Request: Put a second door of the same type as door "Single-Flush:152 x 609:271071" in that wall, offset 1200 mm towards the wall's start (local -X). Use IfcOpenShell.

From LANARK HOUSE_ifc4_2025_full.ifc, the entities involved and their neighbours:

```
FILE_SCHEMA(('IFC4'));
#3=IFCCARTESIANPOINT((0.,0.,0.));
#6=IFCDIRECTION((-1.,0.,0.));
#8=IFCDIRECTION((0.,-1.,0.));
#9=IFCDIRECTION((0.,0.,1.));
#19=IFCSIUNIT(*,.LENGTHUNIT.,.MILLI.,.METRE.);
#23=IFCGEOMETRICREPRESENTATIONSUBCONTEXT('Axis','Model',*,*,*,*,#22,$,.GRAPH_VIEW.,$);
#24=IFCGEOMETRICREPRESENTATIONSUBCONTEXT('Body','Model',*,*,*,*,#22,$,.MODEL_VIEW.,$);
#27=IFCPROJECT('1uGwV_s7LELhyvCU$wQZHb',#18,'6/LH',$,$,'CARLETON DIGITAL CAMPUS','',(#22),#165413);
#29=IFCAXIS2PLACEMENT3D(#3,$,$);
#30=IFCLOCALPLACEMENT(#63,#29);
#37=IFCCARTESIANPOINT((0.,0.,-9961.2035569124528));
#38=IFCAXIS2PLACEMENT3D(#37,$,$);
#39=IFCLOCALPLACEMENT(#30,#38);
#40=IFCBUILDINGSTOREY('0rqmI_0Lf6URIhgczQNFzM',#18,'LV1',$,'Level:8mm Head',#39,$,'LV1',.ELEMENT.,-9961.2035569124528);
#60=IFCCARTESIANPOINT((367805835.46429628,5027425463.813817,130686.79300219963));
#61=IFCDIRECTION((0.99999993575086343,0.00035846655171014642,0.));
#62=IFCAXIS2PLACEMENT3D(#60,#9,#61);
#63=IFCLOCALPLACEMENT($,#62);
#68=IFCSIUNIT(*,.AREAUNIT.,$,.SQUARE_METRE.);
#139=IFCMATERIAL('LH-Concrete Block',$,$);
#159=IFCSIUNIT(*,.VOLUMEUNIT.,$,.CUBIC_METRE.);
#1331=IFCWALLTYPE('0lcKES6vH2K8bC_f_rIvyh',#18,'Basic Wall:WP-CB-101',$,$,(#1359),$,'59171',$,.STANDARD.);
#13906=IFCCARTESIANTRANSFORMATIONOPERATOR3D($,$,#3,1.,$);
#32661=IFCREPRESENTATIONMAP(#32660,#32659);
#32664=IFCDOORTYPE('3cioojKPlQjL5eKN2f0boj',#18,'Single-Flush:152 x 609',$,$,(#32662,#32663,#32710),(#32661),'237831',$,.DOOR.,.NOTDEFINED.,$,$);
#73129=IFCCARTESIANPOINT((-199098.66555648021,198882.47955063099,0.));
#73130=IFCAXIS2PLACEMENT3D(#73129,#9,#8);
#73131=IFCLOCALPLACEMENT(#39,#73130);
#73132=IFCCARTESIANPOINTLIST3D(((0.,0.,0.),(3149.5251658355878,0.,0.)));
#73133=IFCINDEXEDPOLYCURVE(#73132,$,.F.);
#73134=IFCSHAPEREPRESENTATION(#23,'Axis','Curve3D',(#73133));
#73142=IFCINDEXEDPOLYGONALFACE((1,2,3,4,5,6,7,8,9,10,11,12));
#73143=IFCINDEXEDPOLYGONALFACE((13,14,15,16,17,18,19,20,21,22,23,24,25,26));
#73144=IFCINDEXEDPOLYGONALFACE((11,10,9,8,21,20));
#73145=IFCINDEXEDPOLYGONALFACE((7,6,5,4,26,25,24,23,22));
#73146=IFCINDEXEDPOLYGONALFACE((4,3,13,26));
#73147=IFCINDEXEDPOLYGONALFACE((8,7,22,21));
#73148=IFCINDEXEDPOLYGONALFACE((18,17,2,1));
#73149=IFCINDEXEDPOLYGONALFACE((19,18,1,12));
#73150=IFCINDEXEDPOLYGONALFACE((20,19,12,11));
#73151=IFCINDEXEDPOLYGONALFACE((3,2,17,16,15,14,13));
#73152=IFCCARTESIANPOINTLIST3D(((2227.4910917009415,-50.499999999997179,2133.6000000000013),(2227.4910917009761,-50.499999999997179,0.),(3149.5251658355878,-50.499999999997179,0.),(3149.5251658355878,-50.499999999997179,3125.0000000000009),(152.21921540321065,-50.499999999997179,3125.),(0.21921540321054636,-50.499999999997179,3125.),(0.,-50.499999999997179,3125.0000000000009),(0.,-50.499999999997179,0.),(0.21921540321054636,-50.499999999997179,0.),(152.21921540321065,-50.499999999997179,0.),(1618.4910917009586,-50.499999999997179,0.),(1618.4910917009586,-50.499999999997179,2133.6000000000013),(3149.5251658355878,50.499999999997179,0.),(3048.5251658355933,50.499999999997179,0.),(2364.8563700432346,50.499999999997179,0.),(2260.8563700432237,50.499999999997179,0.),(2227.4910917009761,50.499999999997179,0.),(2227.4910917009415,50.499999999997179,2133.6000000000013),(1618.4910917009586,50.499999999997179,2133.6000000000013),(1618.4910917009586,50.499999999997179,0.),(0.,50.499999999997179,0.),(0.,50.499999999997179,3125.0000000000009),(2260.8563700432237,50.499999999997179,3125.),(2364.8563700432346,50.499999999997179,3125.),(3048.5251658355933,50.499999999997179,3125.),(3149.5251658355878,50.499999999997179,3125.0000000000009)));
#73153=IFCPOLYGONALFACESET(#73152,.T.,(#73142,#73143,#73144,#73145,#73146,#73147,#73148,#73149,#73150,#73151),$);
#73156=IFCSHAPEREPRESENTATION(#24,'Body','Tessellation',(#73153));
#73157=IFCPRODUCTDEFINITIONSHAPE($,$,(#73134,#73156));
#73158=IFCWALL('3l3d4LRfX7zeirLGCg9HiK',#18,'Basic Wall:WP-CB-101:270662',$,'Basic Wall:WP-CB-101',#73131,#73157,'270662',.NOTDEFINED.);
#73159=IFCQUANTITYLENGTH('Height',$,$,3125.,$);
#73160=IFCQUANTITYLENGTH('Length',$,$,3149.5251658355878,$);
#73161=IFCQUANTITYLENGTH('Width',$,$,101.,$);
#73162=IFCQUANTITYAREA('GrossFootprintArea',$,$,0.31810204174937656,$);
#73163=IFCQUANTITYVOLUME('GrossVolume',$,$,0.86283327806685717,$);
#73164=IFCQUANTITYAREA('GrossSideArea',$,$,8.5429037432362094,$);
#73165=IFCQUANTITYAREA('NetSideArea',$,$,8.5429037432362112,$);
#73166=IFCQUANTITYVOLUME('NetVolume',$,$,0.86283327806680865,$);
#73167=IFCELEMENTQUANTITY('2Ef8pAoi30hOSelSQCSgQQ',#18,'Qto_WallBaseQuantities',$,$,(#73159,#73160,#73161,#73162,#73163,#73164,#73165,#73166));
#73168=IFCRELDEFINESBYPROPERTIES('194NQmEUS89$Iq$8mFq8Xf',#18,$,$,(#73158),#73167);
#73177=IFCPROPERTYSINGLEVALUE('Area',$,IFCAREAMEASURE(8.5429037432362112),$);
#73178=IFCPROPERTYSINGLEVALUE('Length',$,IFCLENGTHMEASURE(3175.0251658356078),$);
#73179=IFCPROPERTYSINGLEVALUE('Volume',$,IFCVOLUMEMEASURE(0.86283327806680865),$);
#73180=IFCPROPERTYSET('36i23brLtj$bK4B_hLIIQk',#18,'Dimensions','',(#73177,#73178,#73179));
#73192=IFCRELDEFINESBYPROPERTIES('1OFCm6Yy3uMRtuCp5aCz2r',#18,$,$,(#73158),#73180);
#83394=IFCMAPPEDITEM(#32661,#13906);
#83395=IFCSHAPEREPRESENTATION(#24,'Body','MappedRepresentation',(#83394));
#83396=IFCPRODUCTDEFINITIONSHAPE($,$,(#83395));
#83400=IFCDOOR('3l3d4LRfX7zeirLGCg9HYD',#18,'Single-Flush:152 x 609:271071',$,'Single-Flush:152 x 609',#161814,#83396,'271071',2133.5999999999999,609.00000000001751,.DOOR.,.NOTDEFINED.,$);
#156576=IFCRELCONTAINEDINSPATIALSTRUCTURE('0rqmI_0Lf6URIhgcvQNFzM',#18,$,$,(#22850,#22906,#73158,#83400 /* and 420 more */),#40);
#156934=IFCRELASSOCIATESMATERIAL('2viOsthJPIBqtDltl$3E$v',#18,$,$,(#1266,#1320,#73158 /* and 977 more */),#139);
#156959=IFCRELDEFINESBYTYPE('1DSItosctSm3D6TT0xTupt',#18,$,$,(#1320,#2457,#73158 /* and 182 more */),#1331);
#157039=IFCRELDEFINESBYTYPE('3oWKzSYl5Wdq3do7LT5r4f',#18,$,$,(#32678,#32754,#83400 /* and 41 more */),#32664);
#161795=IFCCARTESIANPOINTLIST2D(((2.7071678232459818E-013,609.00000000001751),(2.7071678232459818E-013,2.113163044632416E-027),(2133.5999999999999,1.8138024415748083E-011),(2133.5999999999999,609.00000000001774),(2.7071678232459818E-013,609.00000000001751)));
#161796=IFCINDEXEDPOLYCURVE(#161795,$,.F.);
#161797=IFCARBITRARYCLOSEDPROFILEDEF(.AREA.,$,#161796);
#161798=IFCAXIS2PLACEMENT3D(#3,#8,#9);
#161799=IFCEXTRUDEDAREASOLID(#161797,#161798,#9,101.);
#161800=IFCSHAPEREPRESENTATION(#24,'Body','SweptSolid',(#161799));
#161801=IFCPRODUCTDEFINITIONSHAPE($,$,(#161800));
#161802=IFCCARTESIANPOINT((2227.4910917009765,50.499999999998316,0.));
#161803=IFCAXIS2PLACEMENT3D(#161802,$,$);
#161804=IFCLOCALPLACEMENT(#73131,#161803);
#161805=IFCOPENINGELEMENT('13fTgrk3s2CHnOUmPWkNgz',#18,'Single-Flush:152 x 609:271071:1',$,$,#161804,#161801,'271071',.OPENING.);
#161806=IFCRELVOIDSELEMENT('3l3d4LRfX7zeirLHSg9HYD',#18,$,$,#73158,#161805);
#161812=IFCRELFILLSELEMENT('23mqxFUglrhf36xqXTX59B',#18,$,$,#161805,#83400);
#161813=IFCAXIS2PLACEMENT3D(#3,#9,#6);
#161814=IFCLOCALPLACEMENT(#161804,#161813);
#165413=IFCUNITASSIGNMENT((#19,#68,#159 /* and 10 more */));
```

```python
import ifcopenshell
import ifcopenshell.api.feature
import ifcopenshell.api.geometry
import ifcopenshell.api.pset
import ifcopenshell.api.root
import ifcopenshell.geom
import ifcopenshell.util.element
import ifcopenshell.util.placement
import ifcopenshell.util.shape
import ifcopenshell.util.unit

model = ifcopenshell.open("LANARK HOUSE_ifc4_2025_full.ifc")
unit_scale = ifcopenshell.util.unit.calculate_unit_scale(model)
area_scale = ifcopenshell.util.unit.calculate_unit_scale(model, "AREAUNIT")
volume_scale = ifcopenshell.util.unit.calculate_unit_scale(model, "VOLUMEUNIT")
settings = ifcopenshell.geom.settings()


def volume(element):
    """Net volume in cubic metres, openings subtracted."""
    shape = ifcopenshell.geom.create_shape(settings, element)
    return ifcopenshell.util.shape.get_volume(shape.geometry)


def reuse_history(source, copy):
    """copy_class also copies each property set's owner history, people and application; keep the originals."""
    for rel in copy.IsDefinedBy:
        if rel.is_a("IfcRelDefinesByProperties") and (history := rel.RelatingPropertyDefinition.OwnerHistory):
            rel.RelatingPropertyDefinition.OwnerHistory = source.OwnerHistory
            ifcopenshell.util.element.remove_deep2(model, history)


door = model.by_guid("3l3d4LRfX7zeirLGCg9HYD")
opening = door.FillsVoids[0].RelatingOpeningElement
wall = opening.VoidsElements[0].RelatingBuildingElement
before = volume(wall)
shift = ifcopenshell.util.placement.get_local_placement(wall.ObjectPlacement)[:3, 0] * -1.2 / unit_scale

# copy_class copies the void relationship, type, container and properties, but no geometry.
new_opening = ifcopenshell.api.root.copy_class(model, product=opening)
new_opening.Representation = ifcopenshell.util.element.copy_deep(
    model, opening.Representation, exclude=["IfcGeometricRepresentationContext", "IfcRepresentationMap"]
)
new_opening.Name = "Single-Flush:152 x 609"
new_opening.Tag = None
reuse_history(opening, new_opening)
new_door = ifcopenshell.api.root.copy_class(model, product=door)
new_door.Representation = ifcopenshell.util.element.copy_deep(
    model, door.Representation, exclude=["IfcGeometricRepresentationContext", "IfcRepresentationMap"]
)
new_door.Name = "Single-Flush:152 x 609"
new_door.Tag = None
reuse_history(door, new_door)
ifcopenshell.api.feature.add_filling(model, opening=new_opening, element=new_door)

for old, new in ((opening, new_opening), (door, new_door)):
    matrix = ifcopenshell.util.placement.get_local_placement(old.ObjectPlacement)
    matrix[:3, 3] += shift
    ifcopenshell.api.geometry.edit_object_placement(model, product=new, matrix=matrix, is_si=False)

after = volume(wall)
thickness = 0.101  # wall thickness in metres

# Update the wall's stored quantities.
qto = model.by_id(ifcopenshell.util.element.get_pset(wall, "Qto_WallBaseQuantities", should_inherit=False)["id"])
ifcopenshell.api.pset.edit_qto(model, qto=qto, properties={
    "NetSideArea": after / thickness / area_scale,
    "NetVolume": after / volume_scale,
})
pset = model.by_id(ifcopenshell.util.element.get_pset(wall, "Dimensions", should_inherit=False)["id"])
ifcopenshell.api.pset.edit_pset(model, pset=pset, properties={
    "Area": model.create_entity("IfcAreaMeasure", after / thickness / area_scale),
    "Volume": model.create_entity("IfcVolumeMeasure", after / volume_scale),
})

print(f"wall volume {before:.3f} -> {after:.3f} m3")

model.write("LANARK HOUSE_ifc4_2025_full_updated.ifc")
```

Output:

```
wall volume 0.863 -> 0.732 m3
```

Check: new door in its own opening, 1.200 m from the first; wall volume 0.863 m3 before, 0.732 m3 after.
